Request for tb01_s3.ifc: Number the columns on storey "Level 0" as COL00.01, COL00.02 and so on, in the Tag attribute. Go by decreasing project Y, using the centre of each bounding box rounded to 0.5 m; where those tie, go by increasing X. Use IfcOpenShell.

First a look at what the model holds.

```python
import ifcopenshell
import ifcopenshell.util.element
import ifcopenshell.util.placement

model = ifcopenshell.open("tb01_s3.ifc")
print(model.schema)
storey = next(s for s in model.by_type("IfcBuildingStorey") if s.Name == "Level 0")
columns = [e for e in ifcopenshell.util.element.get_decomposition(storey) if e.is_a("IfcColumn")]
for e in sorted(columns, key=lambda e: e.id()):
    origin = ifcopenshell.util.placement.get_local_placement(e.ObjectPlacement)[:3, 3]
    print(e.id(), e.Tag, e.Name, origin.round(2) + 0.0, sep=" | ")
```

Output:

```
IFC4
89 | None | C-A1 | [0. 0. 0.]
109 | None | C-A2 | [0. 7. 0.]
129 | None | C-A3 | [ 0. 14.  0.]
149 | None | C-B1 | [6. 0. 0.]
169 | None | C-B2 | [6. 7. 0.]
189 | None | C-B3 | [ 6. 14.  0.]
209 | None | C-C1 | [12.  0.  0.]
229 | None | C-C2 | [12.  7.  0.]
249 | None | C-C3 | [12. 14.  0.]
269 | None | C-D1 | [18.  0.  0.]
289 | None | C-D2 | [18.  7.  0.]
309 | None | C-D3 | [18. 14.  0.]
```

```python
import ifcopenshell
import ifcopenshell.geom
import ifcopenshell.util.element
import ifcopenshell.util.shape

model = ifcopenshell.open("tb01_s3.ifc")
settings = ifcopenshell.geom.settings()
settings.set("use-world-coords", True)


def centre(element):
    shape = ifcopenshell.geom.create_shape(settings, element)
    return ifcopenshell.util.shape.get_bbox_centroid(shape.geometry)


storey = next(s for s in model.by_type("IfcBuildingStorey") if s.Name == "Level 0")
columns = [e for e in ifcopenshell.util.element.get_decomposition(storey) if e.is_a("IfcColumn")]

# Insertion points can sit at a corner or the storey origin, so sort by the geometry (in metres).
centres = {e: centre(e) for e in columns}
columns.sort(key=lambda e: (-round(centres[e][1] / 0.5), centres[e][0]))

for i, e in enumerate(columns, start=1):
    number = f"COL00.{i:02d}"
    e.Tag = number
    print(e.id(), number)

model.write("tb01_s3_updated.ifc")
```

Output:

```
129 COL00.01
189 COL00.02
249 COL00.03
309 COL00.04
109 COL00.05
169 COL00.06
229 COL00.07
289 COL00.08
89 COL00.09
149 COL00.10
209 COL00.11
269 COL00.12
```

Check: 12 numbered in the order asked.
